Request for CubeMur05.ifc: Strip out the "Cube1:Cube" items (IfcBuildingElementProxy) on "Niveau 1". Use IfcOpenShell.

First a look at what the model holds.

```python
import ifcopenshell
import ifcopenshell.util.element

model = ifcopenshell.open("CubeMur05.ifc")
print(model.schema)
storey = next(s for s in model.by_type("IfcBuildingStorey") if s.Name == "Niveau 1")
proxies = [e for e in ifcopenshell.util.element.get_decomposition(storey) if e.is_a("IfcBuildingElementProxy")]
seen = {}
for e in proxies:
    element_type = ifcopenshell.util.element.get_type(e)
    name = element_type.Name if element_type not in (None, e) else None
    seen[name] = seen.get(name, 0) + 1
for name, count in sorted(seen.items(), key=str):
    print(count, "x", name)
```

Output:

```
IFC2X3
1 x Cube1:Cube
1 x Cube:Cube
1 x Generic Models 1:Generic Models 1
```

```python
import ifcopenshell
import ifcopenshell.api.root
import ifcopenshell.util.element

model = ifcopenshell.open("CubeMur05.ifc")

storey = next(s for s in model.by_type("IfcBuildingStorey") if s.Name == "Niveau 1")
proxies = [e for e in ifcopenshell.util.element.get_decomposition(storey) if e.is_a("IfcBuildingElementProxy")]
targets = [e for e in proxies if (t := ifcopenshell.util.element.get_type(e)) not in (None, e) and t.Name == "Cube1:Cube"]

for e in targets:
    ifcopenshell.api.root.remove_product(model, product=e)
print(len(targets), "removed")

model.write("CubeMur05_v2.ifc")
```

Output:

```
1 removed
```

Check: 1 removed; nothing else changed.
